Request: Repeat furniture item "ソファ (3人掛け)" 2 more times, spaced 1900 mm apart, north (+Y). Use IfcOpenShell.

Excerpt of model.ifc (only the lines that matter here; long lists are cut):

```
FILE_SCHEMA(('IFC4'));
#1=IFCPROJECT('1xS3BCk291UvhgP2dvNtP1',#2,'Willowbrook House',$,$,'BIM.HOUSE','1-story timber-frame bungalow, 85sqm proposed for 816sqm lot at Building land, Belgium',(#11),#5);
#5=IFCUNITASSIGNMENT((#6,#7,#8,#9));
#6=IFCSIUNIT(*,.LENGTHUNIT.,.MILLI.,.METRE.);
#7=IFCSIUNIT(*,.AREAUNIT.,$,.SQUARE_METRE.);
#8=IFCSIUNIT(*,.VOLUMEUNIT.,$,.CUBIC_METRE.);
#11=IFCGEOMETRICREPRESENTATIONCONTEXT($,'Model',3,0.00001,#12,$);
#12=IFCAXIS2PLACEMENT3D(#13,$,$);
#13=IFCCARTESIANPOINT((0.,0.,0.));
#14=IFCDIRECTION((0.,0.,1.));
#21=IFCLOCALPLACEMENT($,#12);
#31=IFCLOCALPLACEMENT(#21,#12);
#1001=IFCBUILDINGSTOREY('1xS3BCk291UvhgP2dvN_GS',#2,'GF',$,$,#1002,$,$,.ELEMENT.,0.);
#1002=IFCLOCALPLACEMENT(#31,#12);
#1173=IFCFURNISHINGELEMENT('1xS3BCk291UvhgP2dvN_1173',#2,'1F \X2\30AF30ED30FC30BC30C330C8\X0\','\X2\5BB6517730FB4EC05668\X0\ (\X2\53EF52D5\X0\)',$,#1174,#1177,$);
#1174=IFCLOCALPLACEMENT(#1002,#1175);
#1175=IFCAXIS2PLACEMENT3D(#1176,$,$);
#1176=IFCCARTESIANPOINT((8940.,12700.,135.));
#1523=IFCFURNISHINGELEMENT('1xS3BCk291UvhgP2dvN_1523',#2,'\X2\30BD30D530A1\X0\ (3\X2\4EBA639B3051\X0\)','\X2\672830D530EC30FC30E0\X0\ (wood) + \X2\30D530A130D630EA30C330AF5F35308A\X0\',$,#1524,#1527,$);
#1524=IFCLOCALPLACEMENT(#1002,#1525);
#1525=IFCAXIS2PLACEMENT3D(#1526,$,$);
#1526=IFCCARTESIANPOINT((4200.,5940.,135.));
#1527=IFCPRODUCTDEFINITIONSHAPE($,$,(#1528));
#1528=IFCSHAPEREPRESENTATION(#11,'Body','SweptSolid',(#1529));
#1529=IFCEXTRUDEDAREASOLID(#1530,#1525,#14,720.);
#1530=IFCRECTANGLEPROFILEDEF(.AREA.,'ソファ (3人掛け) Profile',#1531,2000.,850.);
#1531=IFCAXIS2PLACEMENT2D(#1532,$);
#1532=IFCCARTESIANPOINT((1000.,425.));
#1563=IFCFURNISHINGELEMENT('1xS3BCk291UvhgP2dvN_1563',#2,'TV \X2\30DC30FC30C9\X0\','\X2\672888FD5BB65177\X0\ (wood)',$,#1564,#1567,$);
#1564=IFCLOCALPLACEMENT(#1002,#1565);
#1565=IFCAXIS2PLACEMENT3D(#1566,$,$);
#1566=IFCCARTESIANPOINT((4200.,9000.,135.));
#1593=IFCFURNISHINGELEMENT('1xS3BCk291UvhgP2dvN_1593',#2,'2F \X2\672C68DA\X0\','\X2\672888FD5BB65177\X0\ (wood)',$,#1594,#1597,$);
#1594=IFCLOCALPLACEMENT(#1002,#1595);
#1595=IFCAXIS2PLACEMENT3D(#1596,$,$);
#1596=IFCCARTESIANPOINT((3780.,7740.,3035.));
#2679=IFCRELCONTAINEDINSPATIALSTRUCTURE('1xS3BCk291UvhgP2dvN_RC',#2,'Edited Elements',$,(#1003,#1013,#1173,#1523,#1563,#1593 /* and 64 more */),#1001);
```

```python
import numpy as np
import ifcopenshell
import ifcopenshell.api.geometry
import ifcopenshell.api.root
import ifcopenshell.util.element
import ifcopenshell.util.placement
import ifcopenshell.util.unit

model = ifcopenshell.open("model.ifc")
unit_scale = ifcopenshell.util.unit.calculate_unit_scale(model)


def reuse_history(source, copy):
    """copy_class also copies each property set's owner history, people and application; keep the originals."""
    for rel in copy.IsDefinedBy:
        if rel.is_a("IfcRelDefinesByProperties") and (history := rel.RelatingPropertyDefinition.OwnerHistory):
            rel.RelatingPropertyDefinition.OwnerHistory = source.OwnerHistory
            ifcopenshell.util.element.remove_deep2(model, history)


source = model.by_id(1523)
base = ifcopenshell.util.placement.get_local_placement(source.ObjectPlacement)
step = np.array([0.0, 1.0, 0.0]) * 1.9 / unit_scale

for i in range(1, 3):
    copy = ifcopenshell.api.root.copy_class(model, product=source)
    copy.Representation = ifcopenshell.util.element.copy_deep(
        model, source.Representation, exclude=["IfcGeometricRepresentationContext", "IfcRepresentationMap"]
    )
    reuse_history(source, copy)
    matrix = base.copy()
    matrix[:3, 3] += i * step
    print("added at", matrix[:3, 3].round(3) + 0.0)
    ifcopenshell.api.geometry.edit_object_placement(model, product=copy, matrix=matrix, is_si=False)

model.write("model_rev.ifc")
```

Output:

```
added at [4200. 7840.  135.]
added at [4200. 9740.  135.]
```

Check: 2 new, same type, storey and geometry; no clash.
